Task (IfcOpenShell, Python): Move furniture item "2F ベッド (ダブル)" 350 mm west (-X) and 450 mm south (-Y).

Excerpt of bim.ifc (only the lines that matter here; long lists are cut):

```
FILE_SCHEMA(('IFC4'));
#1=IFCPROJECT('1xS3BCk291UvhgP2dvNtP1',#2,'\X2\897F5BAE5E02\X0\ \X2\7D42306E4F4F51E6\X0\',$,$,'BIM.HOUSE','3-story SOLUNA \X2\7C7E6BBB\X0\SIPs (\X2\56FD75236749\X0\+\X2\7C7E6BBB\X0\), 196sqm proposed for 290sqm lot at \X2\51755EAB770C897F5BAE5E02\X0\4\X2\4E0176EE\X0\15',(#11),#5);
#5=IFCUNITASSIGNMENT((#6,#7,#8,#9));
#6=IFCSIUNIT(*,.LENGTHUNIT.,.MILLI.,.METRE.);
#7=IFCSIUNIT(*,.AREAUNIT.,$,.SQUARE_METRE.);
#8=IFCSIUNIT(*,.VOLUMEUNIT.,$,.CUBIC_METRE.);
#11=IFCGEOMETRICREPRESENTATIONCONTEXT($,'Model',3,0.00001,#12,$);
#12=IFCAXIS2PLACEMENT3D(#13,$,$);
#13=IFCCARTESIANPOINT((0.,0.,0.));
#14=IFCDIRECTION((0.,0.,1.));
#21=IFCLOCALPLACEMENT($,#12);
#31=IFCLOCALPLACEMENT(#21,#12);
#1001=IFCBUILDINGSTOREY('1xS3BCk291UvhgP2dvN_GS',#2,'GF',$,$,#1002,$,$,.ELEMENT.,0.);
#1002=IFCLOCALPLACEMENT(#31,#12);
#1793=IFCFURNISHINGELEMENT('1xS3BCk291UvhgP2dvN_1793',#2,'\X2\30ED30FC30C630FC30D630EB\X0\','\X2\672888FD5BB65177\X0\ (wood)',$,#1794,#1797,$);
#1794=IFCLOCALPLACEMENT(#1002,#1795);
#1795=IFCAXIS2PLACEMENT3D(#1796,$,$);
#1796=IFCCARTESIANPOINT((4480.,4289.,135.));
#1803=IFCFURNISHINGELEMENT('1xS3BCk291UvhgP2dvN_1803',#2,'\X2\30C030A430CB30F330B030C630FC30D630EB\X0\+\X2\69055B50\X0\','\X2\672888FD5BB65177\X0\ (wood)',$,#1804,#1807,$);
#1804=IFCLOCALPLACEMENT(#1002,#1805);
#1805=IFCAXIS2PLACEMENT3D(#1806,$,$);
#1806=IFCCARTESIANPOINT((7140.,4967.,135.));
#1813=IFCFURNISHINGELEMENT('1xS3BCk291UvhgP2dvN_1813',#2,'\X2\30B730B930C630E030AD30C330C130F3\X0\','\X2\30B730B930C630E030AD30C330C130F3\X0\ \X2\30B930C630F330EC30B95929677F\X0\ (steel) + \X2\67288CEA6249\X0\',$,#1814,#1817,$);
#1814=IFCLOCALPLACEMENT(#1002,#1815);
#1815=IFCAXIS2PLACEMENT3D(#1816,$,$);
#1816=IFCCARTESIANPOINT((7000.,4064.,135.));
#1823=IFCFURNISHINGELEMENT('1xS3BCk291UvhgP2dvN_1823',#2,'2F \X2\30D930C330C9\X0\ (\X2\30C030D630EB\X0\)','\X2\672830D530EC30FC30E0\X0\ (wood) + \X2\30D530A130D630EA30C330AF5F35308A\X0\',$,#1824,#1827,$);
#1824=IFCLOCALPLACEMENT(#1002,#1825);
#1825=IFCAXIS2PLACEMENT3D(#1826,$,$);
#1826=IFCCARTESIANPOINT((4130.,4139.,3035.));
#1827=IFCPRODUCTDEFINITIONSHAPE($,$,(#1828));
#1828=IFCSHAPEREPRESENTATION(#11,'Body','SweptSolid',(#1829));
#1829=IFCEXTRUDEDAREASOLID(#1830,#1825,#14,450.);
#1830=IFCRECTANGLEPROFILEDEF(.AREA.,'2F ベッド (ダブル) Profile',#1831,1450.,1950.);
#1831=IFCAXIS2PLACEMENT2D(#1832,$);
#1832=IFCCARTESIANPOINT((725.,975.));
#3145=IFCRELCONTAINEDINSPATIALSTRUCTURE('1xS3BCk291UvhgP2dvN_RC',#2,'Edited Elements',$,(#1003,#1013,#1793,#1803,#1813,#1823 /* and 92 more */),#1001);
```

```python
import ifcopenshell
import ifcopenshell.api.geometry
import ifcopenshell.util.placement

model = ifcopenshell.open("bim.ifc")

item = model.by_guid("1xS3BCk291UvhgP2dvN_1823")
matrix = ifcopenshell.util.placement.get_local_placement(item.ObjectPlacement)
matrix[0, 3] -= 350.0
matrix[1, 3] -= 450.0
ifcopenshell.api.geometry.edit_object_placement(model, product=item, matrix=matrix, is_si=False)

print(ifcopenshell.util.placement.get_local_placement(item.ObjectPlacement).round(3) + 0.0)

model.write("bim-out.ifc")
```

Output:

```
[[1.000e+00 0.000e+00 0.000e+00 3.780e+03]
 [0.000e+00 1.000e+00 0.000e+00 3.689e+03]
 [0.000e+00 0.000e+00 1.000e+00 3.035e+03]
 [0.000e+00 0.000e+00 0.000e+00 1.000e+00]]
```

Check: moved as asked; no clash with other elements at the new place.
